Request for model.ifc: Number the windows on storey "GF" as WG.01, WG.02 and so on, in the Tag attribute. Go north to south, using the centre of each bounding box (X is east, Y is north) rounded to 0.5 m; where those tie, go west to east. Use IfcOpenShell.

First a look at what the model holds.

```python
import ifcopenshell
import ifcopenshell.util.element
import ifcopenshell.util.placement

model = ifcopenshell.open("model.ifc")
print(model.schema)
storey = next(s for s in model.by_type("IfcBuildingStorey") if s.Name == "GF")
windows = [e for e in ifcopenshell.util.element.get_decomposition(storey) if e.is_a("IfcWindow")]
for e in sorted(windows, key=lambda e: e.id()):
    origin = ifcopenshell.util.placement.get_local_placement(e.ObjectPlacement)[:3, 3]
    print(e.id(), e.Tag, e.Name, origin.round(2) + 0.0, sep=" | ")
```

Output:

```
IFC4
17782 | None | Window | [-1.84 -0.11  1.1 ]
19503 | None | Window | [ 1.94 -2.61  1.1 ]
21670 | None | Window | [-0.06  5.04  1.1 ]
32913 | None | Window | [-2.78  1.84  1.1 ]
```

```python
import ifcopenshell
import ifcopenshell.geom
import ifcopenshell.util.element
import ifcopenshell.util.shape

model = ifcopenshell.open("model.ifc")
settings = ifcopenshell.geom.settings()
settings.set("use-world-coords", True)


def centre(element):
    shape = ifcopenshell.geom.create_shape(settings, element)
    return ifcopenshell.util.shape.get_bbox_centroid(shape.geometry)


storey = next(s for s in model.by_type("IfcBuildingStorey") if s.Name == "GF")
windows = [e for e in ifcopenshell.util.element.get_decomposition(storey) if e.is_a("IfcWindow")]

# Insertion points can sit at a corner or the storey origin, so sort by the geometry (in metres).
centres = {e: centre(e) for e in windows}
windows.sort(key=lambda e: (-round(centres[e][1] / 0.5), centres[e][0]))

for i, e in enumerate(windows, start=1):
    number = f"WG.{i:02d}"
    e.Tag = number
    print(e.id(), number)

model.write("model_v2.ifc")
```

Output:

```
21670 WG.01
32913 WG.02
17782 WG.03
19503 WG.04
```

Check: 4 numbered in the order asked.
